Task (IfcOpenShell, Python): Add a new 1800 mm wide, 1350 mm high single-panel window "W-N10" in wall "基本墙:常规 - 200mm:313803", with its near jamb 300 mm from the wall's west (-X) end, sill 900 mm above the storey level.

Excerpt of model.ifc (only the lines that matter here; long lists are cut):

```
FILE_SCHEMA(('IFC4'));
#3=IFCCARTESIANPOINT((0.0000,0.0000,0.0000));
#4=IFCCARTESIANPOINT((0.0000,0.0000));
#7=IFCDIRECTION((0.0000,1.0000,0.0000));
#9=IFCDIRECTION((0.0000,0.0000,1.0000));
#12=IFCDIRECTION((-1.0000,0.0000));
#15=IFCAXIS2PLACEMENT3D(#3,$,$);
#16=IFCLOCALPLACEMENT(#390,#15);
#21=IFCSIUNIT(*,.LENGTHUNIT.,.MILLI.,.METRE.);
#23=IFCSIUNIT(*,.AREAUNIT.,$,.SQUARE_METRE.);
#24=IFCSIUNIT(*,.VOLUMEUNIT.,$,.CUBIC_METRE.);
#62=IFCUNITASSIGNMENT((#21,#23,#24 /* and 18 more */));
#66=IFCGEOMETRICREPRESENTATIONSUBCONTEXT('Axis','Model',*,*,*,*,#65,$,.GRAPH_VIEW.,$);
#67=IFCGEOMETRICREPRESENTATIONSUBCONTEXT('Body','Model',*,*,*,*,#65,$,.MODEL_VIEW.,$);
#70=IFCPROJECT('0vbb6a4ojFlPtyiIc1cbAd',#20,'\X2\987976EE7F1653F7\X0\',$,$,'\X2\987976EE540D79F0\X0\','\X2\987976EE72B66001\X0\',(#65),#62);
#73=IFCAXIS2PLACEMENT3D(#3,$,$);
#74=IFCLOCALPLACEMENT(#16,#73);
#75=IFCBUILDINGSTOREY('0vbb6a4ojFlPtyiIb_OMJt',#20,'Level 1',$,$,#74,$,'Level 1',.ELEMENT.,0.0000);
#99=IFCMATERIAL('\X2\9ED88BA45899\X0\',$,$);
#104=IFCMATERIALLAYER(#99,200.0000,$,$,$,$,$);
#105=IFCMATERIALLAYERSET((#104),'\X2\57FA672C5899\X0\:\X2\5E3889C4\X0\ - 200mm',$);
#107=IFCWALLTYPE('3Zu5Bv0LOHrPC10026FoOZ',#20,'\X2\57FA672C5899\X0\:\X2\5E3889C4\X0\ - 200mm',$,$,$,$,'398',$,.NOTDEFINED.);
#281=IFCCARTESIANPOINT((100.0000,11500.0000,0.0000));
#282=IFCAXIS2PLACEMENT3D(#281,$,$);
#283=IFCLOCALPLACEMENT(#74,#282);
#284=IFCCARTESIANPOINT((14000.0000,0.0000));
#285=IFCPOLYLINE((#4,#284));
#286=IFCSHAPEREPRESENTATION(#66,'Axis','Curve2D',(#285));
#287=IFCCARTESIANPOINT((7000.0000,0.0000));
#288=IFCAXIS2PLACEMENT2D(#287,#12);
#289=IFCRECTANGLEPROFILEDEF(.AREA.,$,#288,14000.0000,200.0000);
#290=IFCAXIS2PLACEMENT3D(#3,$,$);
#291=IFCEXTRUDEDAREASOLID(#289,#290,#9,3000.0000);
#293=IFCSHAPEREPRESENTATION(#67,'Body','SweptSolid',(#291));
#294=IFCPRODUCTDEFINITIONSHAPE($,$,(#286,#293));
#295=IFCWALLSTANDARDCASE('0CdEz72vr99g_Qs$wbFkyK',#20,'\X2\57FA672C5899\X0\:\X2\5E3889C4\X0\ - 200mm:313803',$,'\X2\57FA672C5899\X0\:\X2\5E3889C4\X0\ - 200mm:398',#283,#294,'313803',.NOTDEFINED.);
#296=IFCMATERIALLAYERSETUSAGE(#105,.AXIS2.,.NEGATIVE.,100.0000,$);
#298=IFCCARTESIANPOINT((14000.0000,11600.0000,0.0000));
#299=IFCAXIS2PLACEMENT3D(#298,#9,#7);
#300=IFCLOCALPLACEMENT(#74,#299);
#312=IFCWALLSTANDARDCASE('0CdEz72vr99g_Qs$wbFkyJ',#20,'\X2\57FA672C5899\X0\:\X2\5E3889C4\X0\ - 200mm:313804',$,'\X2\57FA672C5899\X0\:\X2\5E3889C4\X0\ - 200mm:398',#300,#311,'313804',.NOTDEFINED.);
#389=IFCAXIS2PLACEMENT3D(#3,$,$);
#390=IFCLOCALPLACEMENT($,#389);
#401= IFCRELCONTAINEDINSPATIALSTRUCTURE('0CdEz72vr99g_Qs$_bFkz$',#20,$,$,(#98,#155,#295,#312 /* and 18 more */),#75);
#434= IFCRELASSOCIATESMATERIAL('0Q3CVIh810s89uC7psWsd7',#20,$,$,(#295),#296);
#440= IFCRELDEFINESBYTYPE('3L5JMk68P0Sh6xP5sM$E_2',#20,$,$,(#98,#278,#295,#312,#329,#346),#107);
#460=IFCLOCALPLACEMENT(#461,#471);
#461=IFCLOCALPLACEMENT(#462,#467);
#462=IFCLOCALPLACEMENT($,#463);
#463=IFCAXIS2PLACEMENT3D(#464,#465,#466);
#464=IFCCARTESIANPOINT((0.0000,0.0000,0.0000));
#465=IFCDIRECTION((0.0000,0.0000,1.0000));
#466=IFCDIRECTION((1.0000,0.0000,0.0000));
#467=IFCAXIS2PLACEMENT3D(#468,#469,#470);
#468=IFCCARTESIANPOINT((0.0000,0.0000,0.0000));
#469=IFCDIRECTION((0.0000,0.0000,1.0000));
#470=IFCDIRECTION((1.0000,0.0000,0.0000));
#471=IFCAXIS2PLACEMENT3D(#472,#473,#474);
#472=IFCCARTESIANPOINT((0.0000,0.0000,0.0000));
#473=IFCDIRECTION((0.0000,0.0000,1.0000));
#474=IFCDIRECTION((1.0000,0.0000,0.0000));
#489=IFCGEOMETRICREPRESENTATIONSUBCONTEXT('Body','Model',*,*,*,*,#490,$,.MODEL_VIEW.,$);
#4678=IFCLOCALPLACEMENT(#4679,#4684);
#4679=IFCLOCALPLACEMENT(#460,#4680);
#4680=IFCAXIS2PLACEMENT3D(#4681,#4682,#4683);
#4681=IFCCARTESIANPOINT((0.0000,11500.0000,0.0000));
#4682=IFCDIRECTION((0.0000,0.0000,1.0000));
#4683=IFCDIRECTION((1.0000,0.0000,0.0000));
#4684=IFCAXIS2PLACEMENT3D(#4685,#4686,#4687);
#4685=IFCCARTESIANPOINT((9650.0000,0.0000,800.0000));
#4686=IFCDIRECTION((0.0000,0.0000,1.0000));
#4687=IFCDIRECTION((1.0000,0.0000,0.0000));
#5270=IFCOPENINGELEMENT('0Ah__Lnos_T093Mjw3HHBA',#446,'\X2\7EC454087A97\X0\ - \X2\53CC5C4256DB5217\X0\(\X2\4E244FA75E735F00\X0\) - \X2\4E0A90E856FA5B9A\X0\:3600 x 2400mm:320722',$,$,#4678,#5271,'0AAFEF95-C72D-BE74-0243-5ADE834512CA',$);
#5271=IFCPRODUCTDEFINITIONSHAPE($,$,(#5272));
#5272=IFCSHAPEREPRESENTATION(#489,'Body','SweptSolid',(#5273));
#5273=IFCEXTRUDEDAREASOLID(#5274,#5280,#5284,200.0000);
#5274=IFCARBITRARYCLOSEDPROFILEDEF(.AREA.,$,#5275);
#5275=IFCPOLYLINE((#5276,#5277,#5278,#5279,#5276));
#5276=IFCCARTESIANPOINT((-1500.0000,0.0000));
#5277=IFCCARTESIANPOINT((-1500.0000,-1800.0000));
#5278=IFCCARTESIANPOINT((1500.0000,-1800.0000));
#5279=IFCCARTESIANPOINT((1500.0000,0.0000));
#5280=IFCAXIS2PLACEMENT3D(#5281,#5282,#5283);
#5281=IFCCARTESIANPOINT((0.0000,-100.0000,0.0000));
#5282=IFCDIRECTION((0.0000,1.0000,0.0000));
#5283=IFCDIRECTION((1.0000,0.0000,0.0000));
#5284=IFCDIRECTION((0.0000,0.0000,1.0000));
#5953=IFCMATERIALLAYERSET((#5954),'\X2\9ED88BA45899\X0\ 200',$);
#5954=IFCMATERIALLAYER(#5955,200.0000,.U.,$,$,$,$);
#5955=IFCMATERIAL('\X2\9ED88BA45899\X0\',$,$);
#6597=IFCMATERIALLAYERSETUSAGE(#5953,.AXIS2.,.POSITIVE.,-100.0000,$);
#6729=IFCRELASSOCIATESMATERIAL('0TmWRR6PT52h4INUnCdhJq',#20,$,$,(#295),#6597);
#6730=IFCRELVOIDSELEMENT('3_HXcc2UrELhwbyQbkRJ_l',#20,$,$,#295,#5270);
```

```python
import numpy as np
import ifcopenshell
import ifcopenshell.api.feature
import ifcopenshell.api.geometry
import ifcopenshell.api.root
import ifcopenshell.api.spatial
import ifcopenshell.geom
import ifcopenshell.util.element
import ifcopenshell.util.placement
import ifcopenshell.util.representation
import ifcopenshell.util.shape
import ifcopenshell.util.unit

model = ifcopenshell.open("model.ifc")
unit_scale = ifcopenshell.util.unit.calculate_unit_scale(model)
settings = ifcopenshell.geom.settings()


def volume(element):
    """Net volume in cubic metres, openings subtracted."""
    shape = ifcopenshell.geom.create_shape(settings, element)
    return ifcopenshell.util.shape.get_volume(shape.geometry)


wall = model.by_guid("0CdEz72vr99g_Qs$wbFkyK")
storey = ifcopenshell.util.element.get_container(wall, ifc_class="IfcBuildingStorey")
context = ifcopenshell.util.representation.get_context(model, "Model", "Body", "MODEL_VIEW")
before = volume(wall)

width, height, from_end, sill = 1.8, 1.35, 0.3, 0.9  # metres

# The wall runs along its own X axis, and the end named is its -X end.
wall_shape = ifcopenshell.geom.create_shape(settings, wall)
x, y, z = ifcopenshell.util.shape.get_vertices(wall_shape.geometry).T
start = x.min() + from_end
face, thickness = float(y.min()), float(y.max() - y.min())
wall_matrix = ifcopenshell.util.placement.get_local_placement(wall.ObjectPlacement)
level = ifcopenshell.util.placement.get_local_placement(storey.ObjectPlacement)[2, 3]


def in_wall(x, y):
    """Placement at x, y metres in the wall's axes, at sill height."""
    matrix = wall_matrix.copy()
    matrix[:, 3] = wall_matrix @ np.array([x / unit_scale, y / unit_scale, 0.0, 1.0])
    matrix[2, 3] = level + sill / unit_scale
    return matrix


# Opening: a box that overshoots both wall faces by 50 mm.
opening = ifcopenshell.api.root.create_entity(model, ifc_class="IfcOpeningElement", predefined_type="OPENING")
box = ifcopenshell.api.geometry.add_wall_representation(
    model, context=context, length=width, height=height, thickness=thickness + 0.1
)
ifcopenshell.api.geometry.assign_representation(model, product=opening, representation=box)
ifcopenshell.api.geometry.edit_object_placement(model, product=opening, matrix=in_wall(start, face - 0.05), is_si=False)
ifcopenshell.api.feature.add_feature(model, feature=opening, element=wall)

window = ifcopenshell.api.root.create_entity(model, ifc_class="IfcWindow", name="W-N10", predefined_type="WINDOW")
window.OverallWidth, window.OverallHeight = width / unit_scale, height / unit_scale
window.PartitioningType = "SINGLE_PANEL"
body = ifcopenshell.api.geometry.add_window_representation(
    model,
    context=context,
    overall_width=window.OverallWidth,
    overall_height=window.OverallHeight,
    partition_type="SINGLE_PANEL",
)
ifcopenshell.api.geometry.assign_representation(model, product=window, representation=body)
ifcopenshell.api.spatial.assign_container(model, products=[window], relating_structure=storey)
ifcopenshell.api.feature.add_filling(model, opening=opening, element=window)

# Centre the window in the wall's thickness.
ifcopenshell.api.geometry.edit_object_placement(model, product=window, matrix=in_wall(start, face), is_si=False)
window_shape = ifcopenshell.geom.create_shape(settings, window)
depth = ifcopenshell.util.shape.get_vertices(window_shape.geometry)[:, 1]
offset = face + thickness / 2 - (depth.min() + depth.max()) / 2
ifcopenshell.api.geometry.edit_object_placement(model, product=window, matrix=in_wall(start, offset), is_si=False)

after = volume(wall)

print(f"wall volume {before:.3f} -> {after:.3f} m3")

model.write("model_rev.ifc")
```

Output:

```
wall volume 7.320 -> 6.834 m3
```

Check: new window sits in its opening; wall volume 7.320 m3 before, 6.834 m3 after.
